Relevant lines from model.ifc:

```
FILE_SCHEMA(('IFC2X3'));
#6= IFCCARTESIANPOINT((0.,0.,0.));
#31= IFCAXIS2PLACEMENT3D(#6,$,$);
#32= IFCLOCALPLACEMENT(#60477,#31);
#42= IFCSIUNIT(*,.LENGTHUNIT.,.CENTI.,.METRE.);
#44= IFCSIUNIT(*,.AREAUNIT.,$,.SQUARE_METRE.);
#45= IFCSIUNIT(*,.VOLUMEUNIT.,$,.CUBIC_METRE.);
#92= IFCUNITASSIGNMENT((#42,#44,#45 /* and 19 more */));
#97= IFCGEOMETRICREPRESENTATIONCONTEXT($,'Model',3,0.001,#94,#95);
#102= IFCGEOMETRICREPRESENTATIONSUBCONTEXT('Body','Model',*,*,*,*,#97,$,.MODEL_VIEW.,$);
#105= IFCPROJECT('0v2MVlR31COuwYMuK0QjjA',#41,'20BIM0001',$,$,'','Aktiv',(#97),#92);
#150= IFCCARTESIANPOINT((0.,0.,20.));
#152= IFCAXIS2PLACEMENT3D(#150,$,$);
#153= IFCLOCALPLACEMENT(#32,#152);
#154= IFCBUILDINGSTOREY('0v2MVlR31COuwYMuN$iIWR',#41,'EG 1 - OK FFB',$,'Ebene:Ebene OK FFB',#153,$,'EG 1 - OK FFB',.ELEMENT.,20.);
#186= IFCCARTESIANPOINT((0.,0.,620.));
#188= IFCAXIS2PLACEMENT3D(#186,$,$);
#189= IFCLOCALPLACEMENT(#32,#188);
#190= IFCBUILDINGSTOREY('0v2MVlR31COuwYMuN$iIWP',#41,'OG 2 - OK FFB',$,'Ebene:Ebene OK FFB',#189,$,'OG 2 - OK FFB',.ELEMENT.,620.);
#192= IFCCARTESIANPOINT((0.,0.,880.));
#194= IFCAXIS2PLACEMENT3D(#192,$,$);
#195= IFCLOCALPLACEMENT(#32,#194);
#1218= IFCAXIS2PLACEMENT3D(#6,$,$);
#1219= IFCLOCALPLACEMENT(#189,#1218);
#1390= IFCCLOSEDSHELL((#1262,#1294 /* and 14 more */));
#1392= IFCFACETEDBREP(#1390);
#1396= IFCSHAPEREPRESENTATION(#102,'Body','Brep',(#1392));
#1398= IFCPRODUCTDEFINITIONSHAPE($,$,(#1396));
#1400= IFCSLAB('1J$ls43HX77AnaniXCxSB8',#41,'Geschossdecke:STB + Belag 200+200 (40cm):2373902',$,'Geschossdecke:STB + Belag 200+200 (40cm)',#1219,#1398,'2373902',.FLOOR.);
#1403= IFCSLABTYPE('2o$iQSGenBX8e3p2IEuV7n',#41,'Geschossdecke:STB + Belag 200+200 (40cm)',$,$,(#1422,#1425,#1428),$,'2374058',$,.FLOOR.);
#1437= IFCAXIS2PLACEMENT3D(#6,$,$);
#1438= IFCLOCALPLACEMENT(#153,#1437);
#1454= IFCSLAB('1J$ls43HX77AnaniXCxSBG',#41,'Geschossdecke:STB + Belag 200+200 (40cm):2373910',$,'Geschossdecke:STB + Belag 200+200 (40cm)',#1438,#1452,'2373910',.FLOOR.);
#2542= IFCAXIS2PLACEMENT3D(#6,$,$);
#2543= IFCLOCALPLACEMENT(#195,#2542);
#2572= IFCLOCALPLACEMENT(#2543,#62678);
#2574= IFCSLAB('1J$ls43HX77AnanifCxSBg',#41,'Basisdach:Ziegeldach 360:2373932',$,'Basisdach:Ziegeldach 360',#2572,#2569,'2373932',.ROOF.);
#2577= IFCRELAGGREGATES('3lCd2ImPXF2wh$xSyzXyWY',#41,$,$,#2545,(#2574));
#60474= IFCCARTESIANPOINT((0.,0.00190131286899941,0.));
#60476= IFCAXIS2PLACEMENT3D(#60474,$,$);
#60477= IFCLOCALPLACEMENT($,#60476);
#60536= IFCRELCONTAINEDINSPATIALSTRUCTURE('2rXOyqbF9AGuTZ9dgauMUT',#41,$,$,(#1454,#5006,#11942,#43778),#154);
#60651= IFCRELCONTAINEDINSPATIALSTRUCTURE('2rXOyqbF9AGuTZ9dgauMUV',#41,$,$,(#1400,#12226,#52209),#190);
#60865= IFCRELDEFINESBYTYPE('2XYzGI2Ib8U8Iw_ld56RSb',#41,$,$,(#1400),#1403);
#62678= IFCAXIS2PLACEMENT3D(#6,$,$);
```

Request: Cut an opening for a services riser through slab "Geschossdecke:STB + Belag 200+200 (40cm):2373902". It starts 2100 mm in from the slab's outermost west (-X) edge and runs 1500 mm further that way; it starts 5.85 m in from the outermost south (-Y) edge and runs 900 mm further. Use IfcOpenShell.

```python
import numpy as np
import ifcopenshell
import ifcopenshell.api.feature
import ifcopenshell.api.geometry
import ifcopenshell.api.root
import ifcopenshell.geom
import ifcopenshell.util.placement
import ifcopenshell.util.representation
import ifcopenshell.util.shape
import ifcopenshell.util.unit

model = ifcopenshell.open("model.ifc")
unit_scale = ifcopenshell.util.unit.calculate_unit_scale(model)
settings = ifcopenshell.geom.settings()


def volume(element):
    """Net volume in cubic metres, openings subtracted."""
    shape = ifcopenshell.geom.create_shape(settings, element)
    return ifcopenshell.util.shape.get_volume(shape.geometry)


slab = model.by_guid("1J$ls43HX77AnaniXCxSB8")
before = volume(slab)

# Extent in the slab's own axes, in metres. The edges named are its -X and -Y sides.
slab_shape = ifcopenshell.geom.create_shape(settings, slab)
vertices = ifcopenshell.util.shape.get_vertices(slab_shape.geometry)
x_min, y_min, bottom = vertices.min(axis=0)
top = vertices[:, 2].max()

opening = ifcopenshell.api.root.create_entity(model, ifc_class="IfcOpeningElement", name="Services riser opening")
context = ifcopenshell.util.representation.get_context(model, "Model", "Body", "MODEL_VIEW")
width, depth = 1.5, 0.9
outline = [(0.0, 0.0), (width, 0.0), (width, depth), (0.0, depth), (0.0, 0.0)]
# Overshoot both faces by 50 mm so the cut is clean.
shape = ifcopenshell.api.geometry.add_slab_representation(
    model, context=context, depth=top - bottom + 0.1, polyline=outline
)
ifcopenshell.api.geometry.assign_representation(model, product=opening, representation=shape)

matrix = ifcopenshell.util.placement.get_local_placement(slab.ObjectPlacement)
matrix[:, 3] = matrix @ np.append(np.array([x_min + 2.1, y_min + 5.85, bottom - 0.05]) / unit_scale, 1.0)
ifcopenshell.api.geometry.edit_object_placement(model, product=opening, matrix=matrix, is_si=False)
ifcopenshell.api.feature.add_feature(model, feature=opening, element=slab)

after = volume(slab)

print(f"slab volume {before:.3f} -> {after:.3f} m3")

model.write("model_v2.ifc")
```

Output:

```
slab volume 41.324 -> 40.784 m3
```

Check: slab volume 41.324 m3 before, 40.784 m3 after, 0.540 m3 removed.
